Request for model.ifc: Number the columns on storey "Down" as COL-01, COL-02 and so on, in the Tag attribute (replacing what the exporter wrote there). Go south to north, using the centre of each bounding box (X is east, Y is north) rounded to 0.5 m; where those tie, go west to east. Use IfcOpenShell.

First a look at what the model holds.

```python
import ifcopenshell
import ifcopenshell.util.element
import ifcopenshell.util.placement

model = ifcopenshell.open("model.ifc")
print(model.schema)
storey = next(s for s in model.by_type("IfcBuildingStorey") if s.Name == "Down")
columns = [e for e in ifcopenshell.util.element.get_decomposition(storey) if e.is_a("IfcColumn")]
for e in sorted(columns, key=lambda e: e.id()):
    origin = ifcopenshell.util.placement.get_local_placement(e.ObjectPlacement)[:3, 3]
    print(e.id(), e.Tag, e.Name, origin.round(2) + 0.0, sep=" | ")
```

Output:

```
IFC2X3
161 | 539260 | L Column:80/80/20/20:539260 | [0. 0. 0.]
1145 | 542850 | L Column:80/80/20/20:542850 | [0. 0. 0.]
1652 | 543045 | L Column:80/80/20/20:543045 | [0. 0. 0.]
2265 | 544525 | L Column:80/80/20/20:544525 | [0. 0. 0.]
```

```python
import ifcopenshell
import ifcopenshell.geom
import ifcopenshell.util.element
import ifcopenshell.util.shape

model = ifcopenshell.open("model.ifc")
settings = ifcopenshell.geom.settings()
settings.set("use-world-coords", True)


def centre(element):
    shape = ifcopenshell.geom.create_shape(settings, element)
    return ifcopenshell.util.shape.get_bbox_centroid(shape.geometry)


storey = next(s for s in model.by_type("IfcBuildingStorey") if s.Name == "Down")
columns = [e for e in ifcopenshell.util.element.get_decomposition(storey) if e.is_a("IfcColumn")]

# Insertion points can sit at a corner or the storey origin, so sort by the geometry (in metres).
centres = {e: centre(e) for e in columns}
columns.sort(key=lambda e: (round(centres[e][1] / 0.5), centres[e][0]))

for i, e in enumerate(columns, start=1):
    number = f"COL-{i:02d}"
    e.Tag = number
    print(e.id(), number)

model.write("model_updated.ifc")
```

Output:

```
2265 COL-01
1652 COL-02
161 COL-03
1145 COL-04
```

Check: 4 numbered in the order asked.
